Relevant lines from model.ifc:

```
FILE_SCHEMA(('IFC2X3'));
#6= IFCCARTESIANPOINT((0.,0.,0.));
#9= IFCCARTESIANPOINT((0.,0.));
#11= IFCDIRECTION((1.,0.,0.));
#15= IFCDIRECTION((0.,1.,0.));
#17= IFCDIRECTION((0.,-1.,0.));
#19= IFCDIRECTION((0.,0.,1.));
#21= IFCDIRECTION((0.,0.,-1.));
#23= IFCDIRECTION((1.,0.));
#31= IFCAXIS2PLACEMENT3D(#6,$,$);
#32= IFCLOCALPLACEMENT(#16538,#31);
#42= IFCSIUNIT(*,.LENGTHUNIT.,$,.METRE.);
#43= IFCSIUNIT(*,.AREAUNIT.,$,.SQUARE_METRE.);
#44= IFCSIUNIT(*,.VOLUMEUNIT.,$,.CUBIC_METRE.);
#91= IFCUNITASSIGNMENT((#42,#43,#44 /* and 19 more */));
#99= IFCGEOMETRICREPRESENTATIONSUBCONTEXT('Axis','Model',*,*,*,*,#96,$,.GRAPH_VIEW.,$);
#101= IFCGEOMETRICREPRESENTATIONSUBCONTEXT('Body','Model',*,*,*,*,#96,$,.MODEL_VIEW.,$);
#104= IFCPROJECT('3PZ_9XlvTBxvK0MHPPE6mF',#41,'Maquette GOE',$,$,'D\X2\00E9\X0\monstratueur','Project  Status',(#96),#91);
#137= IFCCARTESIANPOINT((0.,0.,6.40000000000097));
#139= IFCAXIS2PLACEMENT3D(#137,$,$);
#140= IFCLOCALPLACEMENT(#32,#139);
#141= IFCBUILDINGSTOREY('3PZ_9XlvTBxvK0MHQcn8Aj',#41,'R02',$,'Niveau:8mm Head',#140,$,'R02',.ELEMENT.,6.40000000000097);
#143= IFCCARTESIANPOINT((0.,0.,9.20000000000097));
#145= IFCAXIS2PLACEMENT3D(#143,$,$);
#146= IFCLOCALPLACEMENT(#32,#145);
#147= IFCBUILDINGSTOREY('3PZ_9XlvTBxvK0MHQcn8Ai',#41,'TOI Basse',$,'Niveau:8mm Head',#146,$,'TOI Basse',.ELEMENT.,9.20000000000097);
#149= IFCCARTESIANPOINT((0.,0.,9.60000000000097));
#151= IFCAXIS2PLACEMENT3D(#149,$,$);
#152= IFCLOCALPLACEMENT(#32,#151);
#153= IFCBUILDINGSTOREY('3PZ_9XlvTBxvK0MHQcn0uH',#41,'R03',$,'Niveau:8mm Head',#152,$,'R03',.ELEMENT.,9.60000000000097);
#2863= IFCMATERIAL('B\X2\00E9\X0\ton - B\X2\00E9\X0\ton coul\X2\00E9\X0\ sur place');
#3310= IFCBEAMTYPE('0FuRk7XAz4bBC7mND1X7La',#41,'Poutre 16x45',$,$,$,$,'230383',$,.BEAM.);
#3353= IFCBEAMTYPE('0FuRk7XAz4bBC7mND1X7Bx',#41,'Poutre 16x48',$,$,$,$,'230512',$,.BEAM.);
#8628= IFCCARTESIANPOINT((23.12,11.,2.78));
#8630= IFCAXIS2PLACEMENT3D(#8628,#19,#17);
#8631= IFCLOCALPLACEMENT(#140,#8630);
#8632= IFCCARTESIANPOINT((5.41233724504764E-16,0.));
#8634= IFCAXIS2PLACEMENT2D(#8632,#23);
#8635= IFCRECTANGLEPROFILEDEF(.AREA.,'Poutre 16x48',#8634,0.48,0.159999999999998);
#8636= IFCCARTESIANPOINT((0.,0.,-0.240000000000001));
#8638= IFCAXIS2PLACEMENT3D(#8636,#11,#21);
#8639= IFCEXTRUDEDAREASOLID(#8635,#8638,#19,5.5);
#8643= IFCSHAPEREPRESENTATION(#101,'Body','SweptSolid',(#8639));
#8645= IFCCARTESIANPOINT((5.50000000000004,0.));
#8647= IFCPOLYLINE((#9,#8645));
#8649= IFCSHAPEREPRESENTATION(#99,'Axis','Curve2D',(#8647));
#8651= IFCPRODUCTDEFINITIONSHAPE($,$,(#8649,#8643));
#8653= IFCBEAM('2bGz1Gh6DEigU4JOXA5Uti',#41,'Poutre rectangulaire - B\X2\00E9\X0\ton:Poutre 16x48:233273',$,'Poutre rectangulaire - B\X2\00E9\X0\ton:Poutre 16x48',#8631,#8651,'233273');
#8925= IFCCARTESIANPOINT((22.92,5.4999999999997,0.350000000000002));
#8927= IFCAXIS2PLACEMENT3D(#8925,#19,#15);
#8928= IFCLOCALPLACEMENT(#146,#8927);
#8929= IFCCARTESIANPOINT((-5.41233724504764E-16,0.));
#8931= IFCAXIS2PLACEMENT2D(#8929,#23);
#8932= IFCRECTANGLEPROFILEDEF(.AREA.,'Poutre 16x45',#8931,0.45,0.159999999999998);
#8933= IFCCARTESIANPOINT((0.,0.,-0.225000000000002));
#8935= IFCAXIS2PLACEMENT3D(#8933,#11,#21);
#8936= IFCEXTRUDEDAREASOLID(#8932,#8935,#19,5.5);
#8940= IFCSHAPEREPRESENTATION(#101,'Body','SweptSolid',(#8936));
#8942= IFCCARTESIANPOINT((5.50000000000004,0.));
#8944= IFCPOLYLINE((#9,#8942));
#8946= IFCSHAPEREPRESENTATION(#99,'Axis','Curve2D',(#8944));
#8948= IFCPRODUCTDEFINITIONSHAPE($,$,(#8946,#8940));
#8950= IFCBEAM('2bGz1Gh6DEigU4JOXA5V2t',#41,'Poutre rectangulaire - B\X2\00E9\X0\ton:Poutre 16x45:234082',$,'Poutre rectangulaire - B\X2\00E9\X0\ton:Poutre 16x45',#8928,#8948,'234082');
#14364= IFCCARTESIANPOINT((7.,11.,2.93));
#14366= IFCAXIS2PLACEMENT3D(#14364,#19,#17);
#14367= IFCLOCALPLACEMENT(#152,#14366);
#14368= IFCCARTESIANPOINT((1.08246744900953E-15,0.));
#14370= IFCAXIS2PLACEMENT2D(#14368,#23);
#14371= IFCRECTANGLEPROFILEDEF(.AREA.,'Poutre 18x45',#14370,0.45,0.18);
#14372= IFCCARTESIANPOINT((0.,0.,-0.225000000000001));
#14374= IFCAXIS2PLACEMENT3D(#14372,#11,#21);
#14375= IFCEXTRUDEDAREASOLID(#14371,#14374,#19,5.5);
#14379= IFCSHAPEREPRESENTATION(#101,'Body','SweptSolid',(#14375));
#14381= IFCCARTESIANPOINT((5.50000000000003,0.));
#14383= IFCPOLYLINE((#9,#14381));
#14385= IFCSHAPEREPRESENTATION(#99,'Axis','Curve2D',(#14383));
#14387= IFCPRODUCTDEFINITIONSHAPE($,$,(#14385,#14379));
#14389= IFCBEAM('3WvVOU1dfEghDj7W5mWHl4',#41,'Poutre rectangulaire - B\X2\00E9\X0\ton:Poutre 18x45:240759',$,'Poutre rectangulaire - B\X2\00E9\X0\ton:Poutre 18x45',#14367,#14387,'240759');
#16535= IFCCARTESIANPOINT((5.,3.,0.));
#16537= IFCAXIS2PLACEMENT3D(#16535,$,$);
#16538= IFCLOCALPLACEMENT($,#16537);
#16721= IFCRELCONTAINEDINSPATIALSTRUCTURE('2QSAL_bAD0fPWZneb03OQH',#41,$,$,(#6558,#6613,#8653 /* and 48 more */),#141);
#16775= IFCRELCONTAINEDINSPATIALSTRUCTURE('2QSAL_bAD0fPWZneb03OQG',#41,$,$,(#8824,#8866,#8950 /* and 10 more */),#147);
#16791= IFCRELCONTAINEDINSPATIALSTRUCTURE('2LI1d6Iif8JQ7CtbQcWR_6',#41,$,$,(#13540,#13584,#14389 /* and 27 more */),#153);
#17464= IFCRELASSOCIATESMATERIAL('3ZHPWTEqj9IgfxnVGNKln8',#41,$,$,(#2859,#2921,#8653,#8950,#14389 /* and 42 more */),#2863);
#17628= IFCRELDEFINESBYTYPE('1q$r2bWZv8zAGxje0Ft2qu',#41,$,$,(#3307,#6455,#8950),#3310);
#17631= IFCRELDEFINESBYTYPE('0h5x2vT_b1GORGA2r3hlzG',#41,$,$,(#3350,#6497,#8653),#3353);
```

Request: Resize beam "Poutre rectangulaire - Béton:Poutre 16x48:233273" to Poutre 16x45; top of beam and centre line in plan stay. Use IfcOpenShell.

```python
import ifcopenshell
import ifcopenshell.api.type
import ifcopenshell.util.element
import ifcopenshell.util.representation

model = ifcopenshell.open("model.ifc")

member = model.by_guid("2bGz1Gh6DEigU4JOXA5Uti")
source = next(p for p in model.by_type("IfcRectangleProfileDef") if p.ProfileName == "Poutre 16x45")

body = ifcopenshell.util.representation.get_representation(member, "Model", "Body")
solid = body.Items[0]
old_profile = solid.SweptArea

# Copy the section's sizes but keep this member's own profile position.
profile = ifcopenshell.util.element.copy(model, source)
# Profiles are centred, so shift by half the change in depth to hold the top.
shift = (old_profile.XDim - profile.XDim) / 2
x, y = old_profile.Position.Location.Coordinates
up = (-1.0, 0.0)  # upwards, in the solid's own plane
location = model.createIfcCartesianPoint((x + up[0] * shift, y + up[1] * shift))
profile.Position = model.createIfcAxis2Placement2D(location, old_profile.Position.RefDirection)
solid.SweptArea = profile
if not model.get_total_inverses(old_profile):
    ifcopenshell.util.element.remove_deep2(model, old_profile)

new_type = model.by_guid("0FuRk7XAz4bBC7mND1X7La")
ifcopenshell.api.type.assign_type(
    model, related_objects=[member], relating_type=new_type, should_map_representations=False
)
member.Name = member.Name.replace("Poutre 16x48", "Poutre 16x45")
member.ObjectType = "Poutre rectangulaire - Béton:Poutre 16x45"

print(solid.SweptArea)

model.write("model_updated.ifc")
```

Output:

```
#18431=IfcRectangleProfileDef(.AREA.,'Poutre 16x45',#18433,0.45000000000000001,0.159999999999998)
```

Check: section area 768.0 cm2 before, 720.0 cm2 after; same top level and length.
